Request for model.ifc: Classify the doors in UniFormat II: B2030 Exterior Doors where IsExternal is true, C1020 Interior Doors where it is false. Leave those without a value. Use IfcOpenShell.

First a look at what the model holds.

```python
import ifcopenshell
import ifcopenshell.util.element

model = ifcopenshell.open("model.ifc")
print(model.schema)
print("classifications:", [c.Name for c in model.by_type("IfcClassification")])
values = [ifcopenshell.util.element.get_pset(e, "Pset_DoorCommon", "IsExternal") for e in model.by_type("IfcDoor")]
for value in (True, False, None):
    print("IsExternal", value, values.count(value))
```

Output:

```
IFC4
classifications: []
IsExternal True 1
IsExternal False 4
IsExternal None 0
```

```python
import ifcopenshell
import ifcopenshell.api.classification
import ifcopenshell.util.element

model = ifcopenshell.open("model.ifc")

system = ifcopenshell.api.classification.add_classification(model, classification="UniFormat II")

doors = model.by_type("IfcDoor")
external = {e: ifcopenshell.util.element.get_pset(e, "Pset_DoorCommon", "IsExternal") for e in doors}
for flag, code, name in ((True, "B2030", "Exterior Doors"), (False, "C1020", "Interior Doors")):
    products = [e for e in doors if external[e] is flag]
    ifcopenshell.api.classification.add_reference(
        model, products=products, classification=system, identification=code, name=name
    )
    print(code, len(products))

model.write("model-out.ifc")
```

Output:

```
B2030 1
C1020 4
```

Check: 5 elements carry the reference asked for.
